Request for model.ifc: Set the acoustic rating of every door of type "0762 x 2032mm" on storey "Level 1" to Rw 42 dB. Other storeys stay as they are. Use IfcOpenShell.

First a look at what the model holds.

```python
import ifcopenshell
import ifcopenshell.util.element

model = ifcopenshell.open("model.ifc")
print(model.schema)
storey = next(s for s in model.by_type("IfcBuildingStorey") if s.Name == "Level 1")
doors = [e for e in ifcopenshell.util.element.get_decomposition(storey) if e.is_a("IfcDoor")]
seen = {}
for e in doors:
    element_type = ifcopenshell.util.element.get_type(e)
    key = (element_type.Name if element_type != e and element_type else None, ifcopenshell.util.element.get_pset(e, "Pset_DoorCommon", "AcousticRating"))
    seen[key] = seen.get(key, 0) + 1
for (name, value), count in sorted(seen.items(), key=str):
    print(count, "x", name, "|", value)
```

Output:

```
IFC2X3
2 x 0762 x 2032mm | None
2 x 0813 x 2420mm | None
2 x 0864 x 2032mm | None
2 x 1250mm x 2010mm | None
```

```python
import ifcopenshell
import ifcopenshell.api.pset
import ifcopenshell.util.element

model = ifcopenshell.open("model.ifc")

storey = next(s for s in model.by_type("IfcBuildingStorey") if s.Name == "Level 1")
doors = [e for e in ifcopenshell.util.element.get_decomposition(storey) if e.is_a("IfcDoor")]

count = 0
for e in doors:
    element_type = ifcopenshell.util.element.get_type(e)
    if element_type in (None, e) or element_type.Name != "0762 x 2032mm":
        continue
    # add_pset returns the element's existing set when there is one.
    pset = ifcopenshell.api.pset.add_pset(model, product=e, name="Pset_DoorCommon")
    ifcopenshell.api.pset.edit_pset(model, pset=pset, properties={"AcousticRating": "Rw 42 dB"})
    count += 1

print(count, "doors updated")

model.write("model_v2.ifc")
```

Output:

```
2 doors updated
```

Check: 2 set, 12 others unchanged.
